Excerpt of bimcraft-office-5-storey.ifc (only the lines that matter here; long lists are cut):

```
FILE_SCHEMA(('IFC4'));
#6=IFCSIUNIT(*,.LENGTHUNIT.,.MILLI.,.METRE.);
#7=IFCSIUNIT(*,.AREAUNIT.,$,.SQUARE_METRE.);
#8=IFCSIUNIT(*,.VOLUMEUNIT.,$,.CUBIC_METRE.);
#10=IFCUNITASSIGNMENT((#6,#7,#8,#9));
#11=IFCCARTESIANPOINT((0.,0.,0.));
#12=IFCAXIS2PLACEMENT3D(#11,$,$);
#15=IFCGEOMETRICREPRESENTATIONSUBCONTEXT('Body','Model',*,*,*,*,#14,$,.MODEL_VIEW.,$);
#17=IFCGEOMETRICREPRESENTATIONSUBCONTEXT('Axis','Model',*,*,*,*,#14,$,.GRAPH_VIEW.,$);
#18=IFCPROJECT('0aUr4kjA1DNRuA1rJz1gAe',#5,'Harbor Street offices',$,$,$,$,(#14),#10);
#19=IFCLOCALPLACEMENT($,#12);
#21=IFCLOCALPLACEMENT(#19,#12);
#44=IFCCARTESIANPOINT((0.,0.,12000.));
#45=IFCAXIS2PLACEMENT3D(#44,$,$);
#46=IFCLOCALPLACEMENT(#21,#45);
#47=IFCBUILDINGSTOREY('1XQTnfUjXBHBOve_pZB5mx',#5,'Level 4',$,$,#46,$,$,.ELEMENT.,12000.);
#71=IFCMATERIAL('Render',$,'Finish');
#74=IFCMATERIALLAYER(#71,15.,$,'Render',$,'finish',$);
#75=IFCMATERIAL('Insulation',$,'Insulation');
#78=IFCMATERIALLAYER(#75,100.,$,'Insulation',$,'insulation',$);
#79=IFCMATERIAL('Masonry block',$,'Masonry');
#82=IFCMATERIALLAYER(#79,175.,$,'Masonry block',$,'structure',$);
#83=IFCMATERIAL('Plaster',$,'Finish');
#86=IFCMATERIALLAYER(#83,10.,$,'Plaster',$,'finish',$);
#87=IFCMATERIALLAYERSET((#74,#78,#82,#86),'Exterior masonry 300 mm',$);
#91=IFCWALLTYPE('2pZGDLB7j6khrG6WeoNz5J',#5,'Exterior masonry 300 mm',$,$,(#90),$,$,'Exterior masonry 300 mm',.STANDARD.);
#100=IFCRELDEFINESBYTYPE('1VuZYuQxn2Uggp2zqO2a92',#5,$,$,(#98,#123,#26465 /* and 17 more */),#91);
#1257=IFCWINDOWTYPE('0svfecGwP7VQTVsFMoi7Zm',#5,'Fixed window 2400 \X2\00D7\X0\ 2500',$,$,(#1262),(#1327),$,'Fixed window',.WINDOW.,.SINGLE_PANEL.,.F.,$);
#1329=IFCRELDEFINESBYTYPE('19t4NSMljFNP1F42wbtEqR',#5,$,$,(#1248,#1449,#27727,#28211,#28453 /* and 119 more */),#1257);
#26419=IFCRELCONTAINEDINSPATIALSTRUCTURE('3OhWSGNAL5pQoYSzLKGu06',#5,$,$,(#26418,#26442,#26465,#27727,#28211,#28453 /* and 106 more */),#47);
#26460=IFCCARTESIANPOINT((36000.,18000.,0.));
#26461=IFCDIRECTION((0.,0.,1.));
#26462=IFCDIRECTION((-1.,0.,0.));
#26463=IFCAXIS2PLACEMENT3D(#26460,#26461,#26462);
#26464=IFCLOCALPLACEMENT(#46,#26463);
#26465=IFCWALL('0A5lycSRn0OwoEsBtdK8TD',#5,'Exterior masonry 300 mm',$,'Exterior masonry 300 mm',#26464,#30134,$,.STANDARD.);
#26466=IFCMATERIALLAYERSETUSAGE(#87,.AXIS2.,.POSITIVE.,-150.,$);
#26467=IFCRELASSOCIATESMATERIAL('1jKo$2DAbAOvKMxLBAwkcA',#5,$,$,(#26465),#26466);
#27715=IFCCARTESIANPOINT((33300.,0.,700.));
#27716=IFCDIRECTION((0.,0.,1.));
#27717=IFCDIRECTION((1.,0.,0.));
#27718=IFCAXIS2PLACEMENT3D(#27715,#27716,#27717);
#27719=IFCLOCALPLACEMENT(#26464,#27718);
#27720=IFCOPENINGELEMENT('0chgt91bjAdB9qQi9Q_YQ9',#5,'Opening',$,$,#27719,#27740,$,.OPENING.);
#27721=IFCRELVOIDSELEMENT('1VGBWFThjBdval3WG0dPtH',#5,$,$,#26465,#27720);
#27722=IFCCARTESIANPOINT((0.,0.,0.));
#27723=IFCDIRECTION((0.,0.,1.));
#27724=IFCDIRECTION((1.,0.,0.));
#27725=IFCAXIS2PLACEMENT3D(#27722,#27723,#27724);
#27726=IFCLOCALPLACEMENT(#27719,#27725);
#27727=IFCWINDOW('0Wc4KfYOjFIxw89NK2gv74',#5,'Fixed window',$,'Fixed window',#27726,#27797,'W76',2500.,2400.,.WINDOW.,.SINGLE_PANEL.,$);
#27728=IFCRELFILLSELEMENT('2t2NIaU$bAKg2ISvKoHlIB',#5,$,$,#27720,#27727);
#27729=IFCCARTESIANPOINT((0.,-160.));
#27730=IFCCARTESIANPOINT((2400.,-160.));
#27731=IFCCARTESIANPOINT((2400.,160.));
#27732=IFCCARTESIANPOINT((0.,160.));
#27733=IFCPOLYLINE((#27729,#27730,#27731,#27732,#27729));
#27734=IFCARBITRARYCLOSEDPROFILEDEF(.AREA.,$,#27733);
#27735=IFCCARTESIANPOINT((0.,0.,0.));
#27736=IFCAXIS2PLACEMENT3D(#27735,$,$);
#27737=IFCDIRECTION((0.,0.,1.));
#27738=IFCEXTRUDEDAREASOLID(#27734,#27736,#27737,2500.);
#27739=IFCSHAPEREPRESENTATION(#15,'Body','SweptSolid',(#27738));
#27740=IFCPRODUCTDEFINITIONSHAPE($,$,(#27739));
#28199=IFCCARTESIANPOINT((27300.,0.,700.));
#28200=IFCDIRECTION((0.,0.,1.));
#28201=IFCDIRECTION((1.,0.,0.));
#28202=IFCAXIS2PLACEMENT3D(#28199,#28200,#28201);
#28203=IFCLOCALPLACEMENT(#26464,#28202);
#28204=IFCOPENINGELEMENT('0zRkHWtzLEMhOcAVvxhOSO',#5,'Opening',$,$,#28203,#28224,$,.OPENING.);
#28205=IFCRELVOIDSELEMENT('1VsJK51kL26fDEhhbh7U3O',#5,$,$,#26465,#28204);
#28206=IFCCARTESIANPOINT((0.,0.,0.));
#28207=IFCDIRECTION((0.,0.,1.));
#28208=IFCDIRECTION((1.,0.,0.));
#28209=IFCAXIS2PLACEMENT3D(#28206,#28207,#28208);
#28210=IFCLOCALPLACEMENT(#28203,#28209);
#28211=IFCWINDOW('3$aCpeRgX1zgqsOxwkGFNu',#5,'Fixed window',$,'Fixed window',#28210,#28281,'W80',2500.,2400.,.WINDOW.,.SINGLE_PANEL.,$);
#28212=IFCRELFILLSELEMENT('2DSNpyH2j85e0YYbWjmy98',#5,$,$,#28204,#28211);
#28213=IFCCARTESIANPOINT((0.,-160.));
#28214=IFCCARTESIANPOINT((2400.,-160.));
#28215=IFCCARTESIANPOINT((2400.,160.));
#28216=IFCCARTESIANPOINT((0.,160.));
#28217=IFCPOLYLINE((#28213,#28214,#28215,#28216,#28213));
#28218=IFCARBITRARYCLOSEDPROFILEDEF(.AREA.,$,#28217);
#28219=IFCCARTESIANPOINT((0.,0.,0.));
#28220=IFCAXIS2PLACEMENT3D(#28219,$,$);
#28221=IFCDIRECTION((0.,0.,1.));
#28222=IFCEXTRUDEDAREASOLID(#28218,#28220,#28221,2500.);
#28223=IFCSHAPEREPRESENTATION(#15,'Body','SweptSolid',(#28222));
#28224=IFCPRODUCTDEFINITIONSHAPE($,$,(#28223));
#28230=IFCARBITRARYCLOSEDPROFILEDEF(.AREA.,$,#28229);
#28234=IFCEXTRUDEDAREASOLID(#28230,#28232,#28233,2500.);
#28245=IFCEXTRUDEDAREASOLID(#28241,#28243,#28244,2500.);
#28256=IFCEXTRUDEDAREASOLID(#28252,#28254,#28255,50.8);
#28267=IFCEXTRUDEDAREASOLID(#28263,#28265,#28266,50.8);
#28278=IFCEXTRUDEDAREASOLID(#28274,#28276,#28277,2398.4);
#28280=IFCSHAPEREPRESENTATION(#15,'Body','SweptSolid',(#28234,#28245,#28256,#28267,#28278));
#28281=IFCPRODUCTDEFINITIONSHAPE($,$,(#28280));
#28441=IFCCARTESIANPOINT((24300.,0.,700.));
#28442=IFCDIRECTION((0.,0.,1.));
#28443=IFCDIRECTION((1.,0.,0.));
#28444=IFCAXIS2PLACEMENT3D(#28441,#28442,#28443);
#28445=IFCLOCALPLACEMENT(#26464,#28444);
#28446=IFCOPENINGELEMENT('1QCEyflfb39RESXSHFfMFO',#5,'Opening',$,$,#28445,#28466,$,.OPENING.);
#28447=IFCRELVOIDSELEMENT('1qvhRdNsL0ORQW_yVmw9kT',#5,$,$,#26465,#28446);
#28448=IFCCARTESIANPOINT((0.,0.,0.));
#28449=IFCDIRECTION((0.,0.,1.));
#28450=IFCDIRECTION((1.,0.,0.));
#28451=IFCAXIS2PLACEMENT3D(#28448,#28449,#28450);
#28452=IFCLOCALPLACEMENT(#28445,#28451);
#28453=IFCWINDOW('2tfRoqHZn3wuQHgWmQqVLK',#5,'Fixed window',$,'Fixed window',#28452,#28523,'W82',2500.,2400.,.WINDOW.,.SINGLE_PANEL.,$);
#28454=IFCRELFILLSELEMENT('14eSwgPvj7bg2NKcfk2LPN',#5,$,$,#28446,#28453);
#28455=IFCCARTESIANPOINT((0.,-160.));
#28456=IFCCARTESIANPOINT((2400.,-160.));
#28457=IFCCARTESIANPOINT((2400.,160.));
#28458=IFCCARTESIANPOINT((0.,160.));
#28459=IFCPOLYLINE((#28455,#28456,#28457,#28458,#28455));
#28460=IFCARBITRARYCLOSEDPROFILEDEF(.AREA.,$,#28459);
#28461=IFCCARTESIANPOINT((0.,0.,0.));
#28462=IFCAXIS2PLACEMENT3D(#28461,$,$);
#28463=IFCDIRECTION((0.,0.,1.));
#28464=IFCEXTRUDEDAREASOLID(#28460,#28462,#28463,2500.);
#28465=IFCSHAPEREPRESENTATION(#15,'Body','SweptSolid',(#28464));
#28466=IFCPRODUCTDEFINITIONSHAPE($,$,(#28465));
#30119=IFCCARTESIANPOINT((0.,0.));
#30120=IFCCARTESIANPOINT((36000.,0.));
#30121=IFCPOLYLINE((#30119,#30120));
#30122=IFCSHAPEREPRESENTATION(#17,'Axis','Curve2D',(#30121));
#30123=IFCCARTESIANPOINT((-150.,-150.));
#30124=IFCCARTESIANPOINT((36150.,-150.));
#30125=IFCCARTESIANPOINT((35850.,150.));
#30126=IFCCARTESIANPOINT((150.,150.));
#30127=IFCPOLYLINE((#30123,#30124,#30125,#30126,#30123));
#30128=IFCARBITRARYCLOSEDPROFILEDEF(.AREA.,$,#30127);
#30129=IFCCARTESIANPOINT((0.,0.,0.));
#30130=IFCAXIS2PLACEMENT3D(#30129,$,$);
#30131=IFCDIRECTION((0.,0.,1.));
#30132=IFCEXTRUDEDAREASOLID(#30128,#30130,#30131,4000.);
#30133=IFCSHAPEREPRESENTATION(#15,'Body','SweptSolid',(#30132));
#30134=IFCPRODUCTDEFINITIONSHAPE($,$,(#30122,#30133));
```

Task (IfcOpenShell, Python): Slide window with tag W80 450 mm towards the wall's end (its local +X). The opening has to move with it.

```python
import ifcopenshell
import ifcopenshell.api.geometry
import ifcopenshell.util.placement
import ifcopenshell.util.unit

model = ifcopenshell.open("bimcraft-office-5-storey.ifc")
unit_scale = ifcopenshell.util.unit.calculate_unit_scale(model)

window = model.by_id(28211)
opening = window.FillsVoids[0].RelatingOpeningElement
wall = opening.VoidsElements[0].RelatingBuildingElement

wall_matrix = ifcopenshell.util.placement.get_local_placement(wall.ObjectPlacement)
shift = wall_matrix[:3, 0] * 0.45 / unit_scale
before = ifcopenshell.util.placement.get_local_placement(window.ObjectPlacement)[:3, 3].copy()

# The window is placed relative to its opening, so it follows when the opening moves.
matrix = ifcopenshell.util.placement.get_local_placement(opening.ObjectPlacement)
matrix[:3, 3] += shift
ifcopenshell.api.geometry.edit_object_placement(
    model, product=opening, matrix=matrix, is_si=False, should_transform_children=True
)

after = ifcopenshell.util.placement.get_local_placement(window.ObjectPlacement)[:3, 3]
print("window moved by", (after - before).round(3) + 0.0)

model.write("bimcraft-office-5-storey_edited.ifc")
```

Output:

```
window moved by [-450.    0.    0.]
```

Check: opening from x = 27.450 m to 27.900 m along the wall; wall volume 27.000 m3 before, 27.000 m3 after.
